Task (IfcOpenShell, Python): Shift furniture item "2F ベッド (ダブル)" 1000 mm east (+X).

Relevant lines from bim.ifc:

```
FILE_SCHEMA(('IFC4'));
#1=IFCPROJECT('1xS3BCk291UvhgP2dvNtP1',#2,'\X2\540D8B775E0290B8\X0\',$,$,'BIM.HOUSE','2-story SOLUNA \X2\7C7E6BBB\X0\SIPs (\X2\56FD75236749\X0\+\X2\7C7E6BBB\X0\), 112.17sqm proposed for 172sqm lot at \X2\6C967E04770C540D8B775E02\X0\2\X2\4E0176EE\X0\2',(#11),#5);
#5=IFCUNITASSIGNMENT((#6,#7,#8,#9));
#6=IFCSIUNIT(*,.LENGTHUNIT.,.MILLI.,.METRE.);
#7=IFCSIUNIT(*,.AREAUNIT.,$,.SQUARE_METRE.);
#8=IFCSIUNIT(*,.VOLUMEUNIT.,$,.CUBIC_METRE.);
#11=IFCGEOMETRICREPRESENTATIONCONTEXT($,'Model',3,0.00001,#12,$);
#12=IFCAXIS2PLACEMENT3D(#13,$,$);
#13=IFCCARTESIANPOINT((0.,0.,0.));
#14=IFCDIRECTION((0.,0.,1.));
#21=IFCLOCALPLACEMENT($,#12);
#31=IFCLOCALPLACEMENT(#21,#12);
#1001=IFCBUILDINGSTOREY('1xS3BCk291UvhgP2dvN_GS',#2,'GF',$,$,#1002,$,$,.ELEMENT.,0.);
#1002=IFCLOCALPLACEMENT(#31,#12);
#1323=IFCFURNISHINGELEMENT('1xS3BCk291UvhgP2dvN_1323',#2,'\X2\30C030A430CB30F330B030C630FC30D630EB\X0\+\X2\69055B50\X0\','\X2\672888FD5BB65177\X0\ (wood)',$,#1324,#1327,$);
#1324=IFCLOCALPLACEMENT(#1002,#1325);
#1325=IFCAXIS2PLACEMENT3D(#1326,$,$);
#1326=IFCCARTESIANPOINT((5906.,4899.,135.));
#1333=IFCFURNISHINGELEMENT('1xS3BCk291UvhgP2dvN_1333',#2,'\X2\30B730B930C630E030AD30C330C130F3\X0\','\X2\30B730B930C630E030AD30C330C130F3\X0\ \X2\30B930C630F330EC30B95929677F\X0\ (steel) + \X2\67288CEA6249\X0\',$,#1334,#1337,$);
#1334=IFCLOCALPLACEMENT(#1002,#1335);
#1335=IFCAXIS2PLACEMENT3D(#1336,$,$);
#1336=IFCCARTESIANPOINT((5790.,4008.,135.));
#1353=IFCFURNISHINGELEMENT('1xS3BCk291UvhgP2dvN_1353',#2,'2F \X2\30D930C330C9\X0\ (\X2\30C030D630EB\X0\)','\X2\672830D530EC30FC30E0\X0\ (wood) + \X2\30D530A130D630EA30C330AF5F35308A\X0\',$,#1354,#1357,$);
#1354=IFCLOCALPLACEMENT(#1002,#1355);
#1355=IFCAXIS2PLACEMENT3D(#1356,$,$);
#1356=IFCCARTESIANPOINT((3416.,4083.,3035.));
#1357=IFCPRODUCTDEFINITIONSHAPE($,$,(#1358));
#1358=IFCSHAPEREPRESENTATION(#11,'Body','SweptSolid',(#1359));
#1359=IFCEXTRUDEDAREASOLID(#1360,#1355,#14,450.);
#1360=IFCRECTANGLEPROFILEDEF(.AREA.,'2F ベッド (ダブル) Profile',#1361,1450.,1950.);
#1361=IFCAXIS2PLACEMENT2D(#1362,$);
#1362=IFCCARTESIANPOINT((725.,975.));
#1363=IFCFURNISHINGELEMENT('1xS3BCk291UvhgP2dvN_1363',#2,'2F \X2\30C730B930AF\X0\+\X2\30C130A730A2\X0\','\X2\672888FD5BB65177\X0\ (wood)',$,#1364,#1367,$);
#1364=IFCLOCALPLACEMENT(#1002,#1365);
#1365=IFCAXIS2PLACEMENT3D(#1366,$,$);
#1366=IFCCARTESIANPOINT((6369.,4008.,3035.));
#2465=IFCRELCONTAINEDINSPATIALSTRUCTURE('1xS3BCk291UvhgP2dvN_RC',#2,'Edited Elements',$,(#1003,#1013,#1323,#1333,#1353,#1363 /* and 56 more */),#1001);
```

```python
import ifcopenshell
import ifcopenshell.api.geometry
import ifcopenshell.util.placement

model = ifcopenshell.open("bim.ifc")

item = model.by_guid("1xS3BCk291UvhgP2dvN_1353")
matrix = ifcopenshell.util.placement.get_local_placement(item.ObjectPlacement)
matrix[0, 3] += 1000.0
ifcopenshell.api.geometry.edit_object_placement(model, product=item, matrix=matrix, is_si=False)

print(ifcopenshell.util.placement.get_local_placement(item.ObjectPlacement).round(3) + 0.0)

model.write("bim_updated.ifc")
```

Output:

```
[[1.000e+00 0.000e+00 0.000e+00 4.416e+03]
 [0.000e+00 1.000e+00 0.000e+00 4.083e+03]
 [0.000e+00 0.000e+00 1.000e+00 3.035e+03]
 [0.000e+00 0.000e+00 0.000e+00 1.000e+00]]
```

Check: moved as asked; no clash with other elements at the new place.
